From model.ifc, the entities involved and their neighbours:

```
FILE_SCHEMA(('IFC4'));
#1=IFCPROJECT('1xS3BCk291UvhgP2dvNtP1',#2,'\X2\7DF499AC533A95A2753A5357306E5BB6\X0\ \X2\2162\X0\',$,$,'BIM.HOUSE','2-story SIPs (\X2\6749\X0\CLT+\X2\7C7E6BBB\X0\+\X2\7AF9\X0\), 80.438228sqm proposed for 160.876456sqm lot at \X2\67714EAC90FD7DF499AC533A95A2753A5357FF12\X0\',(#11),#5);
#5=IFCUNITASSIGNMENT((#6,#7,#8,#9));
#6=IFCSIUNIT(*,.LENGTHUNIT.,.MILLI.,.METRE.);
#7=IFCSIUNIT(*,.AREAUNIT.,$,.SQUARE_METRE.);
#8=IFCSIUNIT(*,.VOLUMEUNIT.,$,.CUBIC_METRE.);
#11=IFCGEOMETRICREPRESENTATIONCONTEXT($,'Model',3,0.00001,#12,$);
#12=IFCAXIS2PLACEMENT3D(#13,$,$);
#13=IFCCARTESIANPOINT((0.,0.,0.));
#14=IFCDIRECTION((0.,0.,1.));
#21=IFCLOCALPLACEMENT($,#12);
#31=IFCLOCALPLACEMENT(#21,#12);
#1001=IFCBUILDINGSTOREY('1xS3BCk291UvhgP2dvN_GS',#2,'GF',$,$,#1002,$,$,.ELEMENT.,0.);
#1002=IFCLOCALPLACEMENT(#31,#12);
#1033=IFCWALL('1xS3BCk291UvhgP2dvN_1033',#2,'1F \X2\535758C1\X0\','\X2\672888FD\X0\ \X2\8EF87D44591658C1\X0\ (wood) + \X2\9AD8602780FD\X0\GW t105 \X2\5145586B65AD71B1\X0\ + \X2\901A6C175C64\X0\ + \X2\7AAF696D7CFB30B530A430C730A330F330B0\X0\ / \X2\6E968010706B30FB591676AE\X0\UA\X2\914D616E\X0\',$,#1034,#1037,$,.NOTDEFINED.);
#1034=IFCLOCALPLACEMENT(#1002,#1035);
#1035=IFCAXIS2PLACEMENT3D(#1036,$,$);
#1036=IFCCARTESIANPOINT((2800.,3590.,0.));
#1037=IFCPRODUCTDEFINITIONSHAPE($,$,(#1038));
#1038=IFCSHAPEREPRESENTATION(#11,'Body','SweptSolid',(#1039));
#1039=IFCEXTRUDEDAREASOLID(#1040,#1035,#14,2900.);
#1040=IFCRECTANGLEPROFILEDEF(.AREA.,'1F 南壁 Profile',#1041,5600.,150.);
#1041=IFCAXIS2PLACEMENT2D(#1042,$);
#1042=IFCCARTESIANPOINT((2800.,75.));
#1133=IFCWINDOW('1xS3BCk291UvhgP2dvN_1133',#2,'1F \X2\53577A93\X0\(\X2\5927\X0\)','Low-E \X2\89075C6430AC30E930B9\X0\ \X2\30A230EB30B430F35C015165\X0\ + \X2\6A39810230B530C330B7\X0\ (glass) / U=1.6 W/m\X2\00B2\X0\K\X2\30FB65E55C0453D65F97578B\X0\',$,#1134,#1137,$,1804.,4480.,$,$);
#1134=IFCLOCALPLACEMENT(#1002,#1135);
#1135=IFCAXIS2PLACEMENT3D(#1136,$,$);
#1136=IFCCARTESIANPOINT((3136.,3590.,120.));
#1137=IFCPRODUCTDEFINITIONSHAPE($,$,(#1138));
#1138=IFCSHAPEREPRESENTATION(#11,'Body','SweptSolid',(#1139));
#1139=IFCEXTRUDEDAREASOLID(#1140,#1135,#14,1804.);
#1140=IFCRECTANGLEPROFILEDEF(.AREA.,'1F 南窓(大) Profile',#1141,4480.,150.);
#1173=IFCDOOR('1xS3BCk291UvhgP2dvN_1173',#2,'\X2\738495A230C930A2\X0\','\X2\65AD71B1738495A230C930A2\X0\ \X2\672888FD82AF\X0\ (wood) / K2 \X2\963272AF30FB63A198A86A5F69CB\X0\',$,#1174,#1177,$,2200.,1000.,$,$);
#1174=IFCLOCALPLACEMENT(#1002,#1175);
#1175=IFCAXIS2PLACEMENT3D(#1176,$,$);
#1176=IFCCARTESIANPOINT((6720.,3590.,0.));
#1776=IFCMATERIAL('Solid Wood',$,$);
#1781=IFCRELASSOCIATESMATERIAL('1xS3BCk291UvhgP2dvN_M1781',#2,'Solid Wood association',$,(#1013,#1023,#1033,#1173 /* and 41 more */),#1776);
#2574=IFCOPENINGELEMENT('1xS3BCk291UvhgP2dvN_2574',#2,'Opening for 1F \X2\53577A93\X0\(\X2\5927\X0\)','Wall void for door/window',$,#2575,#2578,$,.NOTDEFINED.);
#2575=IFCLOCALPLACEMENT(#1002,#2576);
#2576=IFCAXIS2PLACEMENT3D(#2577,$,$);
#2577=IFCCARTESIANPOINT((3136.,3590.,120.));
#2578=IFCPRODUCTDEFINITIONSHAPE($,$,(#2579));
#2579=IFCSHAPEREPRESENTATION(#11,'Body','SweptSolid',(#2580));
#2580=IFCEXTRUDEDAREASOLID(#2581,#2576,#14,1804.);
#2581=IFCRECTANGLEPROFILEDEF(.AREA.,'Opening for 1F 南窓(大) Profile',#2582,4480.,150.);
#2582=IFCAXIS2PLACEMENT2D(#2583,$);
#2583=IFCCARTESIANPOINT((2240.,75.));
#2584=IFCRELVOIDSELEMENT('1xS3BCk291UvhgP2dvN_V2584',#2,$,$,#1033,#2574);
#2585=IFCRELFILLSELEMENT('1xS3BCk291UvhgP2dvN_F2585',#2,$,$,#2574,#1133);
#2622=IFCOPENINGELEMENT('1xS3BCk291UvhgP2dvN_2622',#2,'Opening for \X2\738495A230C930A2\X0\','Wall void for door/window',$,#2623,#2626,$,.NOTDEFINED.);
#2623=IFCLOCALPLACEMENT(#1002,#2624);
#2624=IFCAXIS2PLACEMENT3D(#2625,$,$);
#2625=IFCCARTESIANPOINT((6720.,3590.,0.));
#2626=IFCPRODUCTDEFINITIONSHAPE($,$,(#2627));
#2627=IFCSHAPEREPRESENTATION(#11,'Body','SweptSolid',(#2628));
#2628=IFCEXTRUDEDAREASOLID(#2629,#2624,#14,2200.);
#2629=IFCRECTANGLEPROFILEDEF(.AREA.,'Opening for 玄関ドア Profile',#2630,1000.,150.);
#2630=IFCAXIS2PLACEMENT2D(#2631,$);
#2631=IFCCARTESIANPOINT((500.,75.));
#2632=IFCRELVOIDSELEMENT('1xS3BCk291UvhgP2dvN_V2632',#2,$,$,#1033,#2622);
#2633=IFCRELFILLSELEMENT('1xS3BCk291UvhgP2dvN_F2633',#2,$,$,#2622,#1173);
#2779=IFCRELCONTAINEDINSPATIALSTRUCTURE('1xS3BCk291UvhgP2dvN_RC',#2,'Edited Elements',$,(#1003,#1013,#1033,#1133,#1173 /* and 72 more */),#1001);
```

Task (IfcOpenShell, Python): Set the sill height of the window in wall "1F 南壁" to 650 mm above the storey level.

```python
import numpy as np
import ifcopenshell
import ifcopenshell.api.geometry
import ifcopenshell.geom
import ifcopenshell.util.element
import ifcopenshell.util.placement
import ifcopenshell.util.shape
import ifcopenshell.util.unit

model = ifcopenshell.open("model.ifc")
unit_scale = ifcopenshell.util.unit.calculate_unit_scale(model)

window = model.by_guid("1xS3BCk291UvhgP2dvN_1133")
opening = window.FillsVoids[0].RelatingOpeningElement
storey = ifcopenshell.util.element.get_container(window, ifc_class="IfcBuildingStorey")
level = ifcopenshell.util.placement.get_local_placement(storey.ObjectPlacement)[2, 3]

# The opening's origin need not be at the sill, so measure its lowest point.
shape = ifcopenshell.geom.create_shape(ifcopenshell.geom.settings(), opening)
bottom = ifcopenshell.util.shape.get_shape_bottom_elevation(shape, shape.geometry) / unit_scale
dz = level + 0.65 / unit_scale - bottom

shift = np.array([0.0, 0.0, dz])
# The window is not placed relative to its opening, so move both.
for product in (opening, window):
    matrix = ifcopenshell.util.placement.get_local_placement(product.ObjectPlacement)
    matrix[:3, 3] += shift
    ifcopenshell.api.geometry.edit_object_placement(model, product=product, matrix=matrix, is_si=False)

print(f"moved by {dz * unit_scale:+.3f} m")

model.write("model_v2.ifc")
```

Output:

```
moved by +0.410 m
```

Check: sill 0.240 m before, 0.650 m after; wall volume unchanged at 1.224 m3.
